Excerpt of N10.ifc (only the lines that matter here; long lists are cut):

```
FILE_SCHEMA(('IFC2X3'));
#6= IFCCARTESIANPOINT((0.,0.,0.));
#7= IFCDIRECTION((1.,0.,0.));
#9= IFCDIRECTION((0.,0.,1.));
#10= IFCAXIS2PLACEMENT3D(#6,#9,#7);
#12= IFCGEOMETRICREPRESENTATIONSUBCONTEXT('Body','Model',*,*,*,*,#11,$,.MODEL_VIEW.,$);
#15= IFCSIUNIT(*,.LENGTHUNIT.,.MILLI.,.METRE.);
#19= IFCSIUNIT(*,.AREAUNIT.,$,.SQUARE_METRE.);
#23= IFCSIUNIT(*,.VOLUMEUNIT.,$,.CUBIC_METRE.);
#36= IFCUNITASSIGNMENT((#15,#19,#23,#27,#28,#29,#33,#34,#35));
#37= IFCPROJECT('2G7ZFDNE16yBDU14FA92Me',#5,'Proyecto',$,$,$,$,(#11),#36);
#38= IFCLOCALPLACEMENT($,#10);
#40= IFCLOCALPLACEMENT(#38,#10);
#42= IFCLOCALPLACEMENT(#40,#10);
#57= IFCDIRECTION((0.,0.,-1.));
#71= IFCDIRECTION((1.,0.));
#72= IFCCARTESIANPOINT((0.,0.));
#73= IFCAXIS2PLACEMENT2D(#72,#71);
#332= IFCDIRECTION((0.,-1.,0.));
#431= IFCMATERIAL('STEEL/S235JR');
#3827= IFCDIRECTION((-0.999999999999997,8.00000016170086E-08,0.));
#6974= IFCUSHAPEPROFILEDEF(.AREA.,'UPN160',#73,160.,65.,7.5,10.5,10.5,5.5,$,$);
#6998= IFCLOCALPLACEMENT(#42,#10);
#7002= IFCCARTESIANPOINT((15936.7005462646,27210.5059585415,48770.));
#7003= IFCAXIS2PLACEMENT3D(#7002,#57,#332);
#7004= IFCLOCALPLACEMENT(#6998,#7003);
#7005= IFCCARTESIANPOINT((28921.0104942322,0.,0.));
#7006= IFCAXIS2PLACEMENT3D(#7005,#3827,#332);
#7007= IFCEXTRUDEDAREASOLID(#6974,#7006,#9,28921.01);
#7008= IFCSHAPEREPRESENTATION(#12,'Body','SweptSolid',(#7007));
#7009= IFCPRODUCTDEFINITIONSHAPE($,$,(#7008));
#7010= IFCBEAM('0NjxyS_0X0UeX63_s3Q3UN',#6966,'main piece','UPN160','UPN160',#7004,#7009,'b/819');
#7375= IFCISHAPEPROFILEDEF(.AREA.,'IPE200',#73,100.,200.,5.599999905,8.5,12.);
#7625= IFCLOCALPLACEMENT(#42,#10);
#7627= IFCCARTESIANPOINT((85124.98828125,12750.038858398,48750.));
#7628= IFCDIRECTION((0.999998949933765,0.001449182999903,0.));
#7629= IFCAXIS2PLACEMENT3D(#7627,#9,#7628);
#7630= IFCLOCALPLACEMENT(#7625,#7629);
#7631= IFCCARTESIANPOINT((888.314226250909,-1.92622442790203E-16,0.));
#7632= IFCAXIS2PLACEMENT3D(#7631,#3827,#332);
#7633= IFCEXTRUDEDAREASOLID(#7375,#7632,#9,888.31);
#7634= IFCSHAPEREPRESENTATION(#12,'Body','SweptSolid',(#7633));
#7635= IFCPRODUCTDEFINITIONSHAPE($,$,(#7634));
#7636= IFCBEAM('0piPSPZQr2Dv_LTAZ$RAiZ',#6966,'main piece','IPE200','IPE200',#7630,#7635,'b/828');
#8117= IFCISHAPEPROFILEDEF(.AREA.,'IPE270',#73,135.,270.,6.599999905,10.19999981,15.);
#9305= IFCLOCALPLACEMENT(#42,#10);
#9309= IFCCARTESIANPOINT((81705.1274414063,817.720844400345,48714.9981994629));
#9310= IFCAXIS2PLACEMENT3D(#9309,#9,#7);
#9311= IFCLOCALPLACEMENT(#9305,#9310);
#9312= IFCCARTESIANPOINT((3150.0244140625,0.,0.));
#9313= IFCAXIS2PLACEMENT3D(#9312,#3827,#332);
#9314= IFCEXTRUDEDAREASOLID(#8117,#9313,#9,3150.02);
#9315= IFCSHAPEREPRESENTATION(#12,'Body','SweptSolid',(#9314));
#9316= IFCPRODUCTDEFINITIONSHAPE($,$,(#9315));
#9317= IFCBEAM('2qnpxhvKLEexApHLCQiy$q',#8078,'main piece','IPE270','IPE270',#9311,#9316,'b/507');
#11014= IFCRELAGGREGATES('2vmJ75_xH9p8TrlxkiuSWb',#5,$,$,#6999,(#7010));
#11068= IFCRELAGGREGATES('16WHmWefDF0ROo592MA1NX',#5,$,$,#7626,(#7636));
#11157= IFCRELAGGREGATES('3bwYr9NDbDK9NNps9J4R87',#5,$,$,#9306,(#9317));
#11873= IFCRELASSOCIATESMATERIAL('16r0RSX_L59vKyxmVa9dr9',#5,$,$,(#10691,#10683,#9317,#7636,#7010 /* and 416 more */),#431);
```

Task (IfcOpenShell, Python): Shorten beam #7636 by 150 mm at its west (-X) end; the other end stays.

```python
import ifcopenshell
import ifcopenshell.util.representation

model = ifcopenshell.open("N10.ifc")

member = model.by_guid("0piPSPZQr2Dv_LTAZ$RAiZ")
change = -150.0

# The extrusion runs towards the end named, so only its depth changes.
body = ifcopenshell.util.representation.get_representation(member, "Model", "Body")
solid = body.Items[0]
old_length = solid.Depth
solid.Depth += change

print(f"length {old_length:g} -> {solid.Depth:g}")

model.write("N10-out.ifc")
```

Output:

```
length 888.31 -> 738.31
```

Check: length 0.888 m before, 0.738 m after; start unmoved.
